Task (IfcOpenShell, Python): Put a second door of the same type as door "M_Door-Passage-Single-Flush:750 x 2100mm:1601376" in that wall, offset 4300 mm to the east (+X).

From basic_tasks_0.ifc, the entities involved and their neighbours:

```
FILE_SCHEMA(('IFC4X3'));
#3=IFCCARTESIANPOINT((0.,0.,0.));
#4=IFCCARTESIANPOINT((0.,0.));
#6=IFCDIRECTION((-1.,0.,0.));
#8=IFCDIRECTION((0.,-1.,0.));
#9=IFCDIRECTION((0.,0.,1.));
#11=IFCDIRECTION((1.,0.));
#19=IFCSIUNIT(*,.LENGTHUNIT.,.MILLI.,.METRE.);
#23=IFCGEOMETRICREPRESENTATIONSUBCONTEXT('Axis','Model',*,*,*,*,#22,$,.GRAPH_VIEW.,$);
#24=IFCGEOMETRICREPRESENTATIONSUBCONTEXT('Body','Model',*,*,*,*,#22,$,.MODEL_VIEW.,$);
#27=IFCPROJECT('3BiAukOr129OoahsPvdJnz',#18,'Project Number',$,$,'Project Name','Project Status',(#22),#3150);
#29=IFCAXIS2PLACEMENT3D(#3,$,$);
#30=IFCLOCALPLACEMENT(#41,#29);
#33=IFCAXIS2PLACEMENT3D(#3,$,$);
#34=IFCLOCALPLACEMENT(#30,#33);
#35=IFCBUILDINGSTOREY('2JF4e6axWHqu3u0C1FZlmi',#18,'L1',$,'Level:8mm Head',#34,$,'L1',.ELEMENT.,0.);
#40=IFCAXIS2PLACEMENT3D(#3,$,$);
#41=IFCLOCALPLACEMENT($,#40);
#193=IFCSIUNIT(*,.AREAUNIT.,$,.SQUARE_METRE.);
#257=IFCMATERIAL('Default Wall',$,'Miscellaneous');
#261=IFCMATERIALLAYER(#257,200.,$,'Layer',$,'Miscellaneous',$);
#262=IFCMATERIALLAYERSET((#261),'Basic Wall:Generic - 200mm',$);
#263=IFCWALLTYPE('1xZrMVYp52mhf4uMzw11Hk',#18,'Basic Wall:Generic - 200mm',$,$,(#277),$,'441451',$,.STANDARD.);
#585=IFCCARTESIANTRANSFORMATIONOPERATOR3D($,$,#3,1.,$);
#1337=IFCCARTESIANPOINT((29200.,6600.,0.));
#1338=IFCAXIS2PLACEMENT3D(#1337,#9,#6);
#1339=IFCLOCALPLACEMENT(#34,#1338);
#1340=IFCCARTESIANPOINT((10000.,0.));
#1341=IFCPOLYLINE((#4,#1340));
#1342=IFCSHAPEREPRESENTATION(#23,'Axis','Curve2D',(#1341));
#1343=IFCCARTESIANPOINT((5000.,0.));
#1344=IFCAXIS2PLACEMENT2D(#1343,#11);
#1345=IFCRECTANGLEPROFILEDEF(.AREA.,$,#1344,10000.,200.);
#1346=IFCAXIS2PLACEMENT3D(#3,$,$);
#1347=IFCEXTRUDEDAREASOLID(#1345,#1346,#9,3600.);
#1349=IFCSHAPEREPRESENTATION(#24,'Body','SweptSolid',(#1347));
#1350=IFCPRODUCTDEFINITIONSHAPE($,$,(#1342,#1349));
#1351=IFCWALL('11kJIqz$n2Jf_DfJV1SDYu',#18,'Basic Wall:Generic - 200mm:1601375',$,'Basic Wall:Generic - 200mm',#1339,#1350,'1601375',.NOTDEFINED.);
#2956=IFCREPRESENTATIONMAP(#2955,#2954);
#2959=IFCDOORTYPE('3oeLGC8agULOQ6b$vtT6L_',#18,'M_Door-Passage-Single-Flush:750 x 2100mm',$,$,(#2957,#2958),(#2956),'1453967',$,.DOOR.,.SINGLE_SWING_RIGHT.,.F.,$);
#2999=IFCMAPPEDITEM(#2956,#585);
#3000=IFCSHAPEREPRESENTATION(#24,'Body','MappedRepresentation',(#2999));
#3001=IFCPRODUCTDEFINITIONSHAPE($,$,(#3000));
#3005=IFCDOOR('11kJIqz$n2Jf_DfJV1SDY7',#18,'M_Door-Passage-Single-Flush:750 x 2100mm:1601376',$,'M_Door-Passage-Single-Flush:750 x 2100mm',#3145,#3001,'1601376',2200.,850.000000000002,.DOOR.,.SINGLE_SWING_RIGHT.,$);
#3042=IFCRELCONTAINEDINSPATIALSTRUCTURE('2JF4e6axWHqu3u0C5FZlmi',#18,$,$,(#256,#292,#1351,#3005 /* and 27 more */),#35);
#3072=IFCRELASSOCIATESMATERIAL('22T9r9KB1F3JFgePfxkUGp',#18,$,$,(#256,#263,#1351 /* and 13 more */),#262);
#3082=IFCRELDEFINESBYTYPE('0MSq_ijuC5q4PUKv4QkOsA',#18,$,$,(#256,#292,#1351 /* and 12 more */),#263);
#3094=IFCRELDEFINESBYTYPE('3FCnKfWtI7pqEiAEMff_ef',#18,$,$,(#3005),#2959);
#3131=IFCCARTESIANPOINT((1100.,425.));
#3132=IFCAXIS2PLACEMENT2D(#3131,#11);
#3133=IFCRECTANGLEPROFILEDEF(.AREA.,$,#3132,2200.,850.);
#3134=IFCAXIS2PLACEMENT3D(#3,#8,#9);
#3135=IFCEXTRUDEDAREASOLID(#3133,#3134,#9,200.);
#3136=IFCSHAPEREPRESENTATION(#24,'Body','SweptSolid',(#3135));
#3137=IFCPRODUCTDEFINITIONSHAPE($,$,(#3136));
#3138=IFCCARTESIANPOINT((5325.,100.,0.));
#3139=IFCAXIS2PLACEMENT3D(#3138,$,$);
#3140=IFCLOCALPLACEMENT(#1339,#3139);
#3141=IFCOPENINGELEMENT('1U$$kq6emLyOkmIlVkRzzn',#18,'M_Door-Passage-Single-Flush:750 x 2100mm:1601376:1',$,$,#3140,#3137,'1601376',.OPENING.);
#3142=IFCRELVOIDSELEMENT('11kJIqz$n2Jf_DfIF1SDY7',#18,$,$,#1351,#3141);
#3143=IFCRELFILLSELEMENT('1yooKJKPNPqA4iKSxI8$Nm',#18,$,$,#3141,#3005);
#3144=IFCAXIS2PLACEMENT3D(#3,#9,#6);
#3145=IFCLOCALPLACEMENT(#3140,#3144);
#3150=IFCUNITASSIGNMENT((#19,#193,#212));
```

```python
import ifcopenshell
import ifcopenshell.api.feature
import ifcopenshell.api.geometry
import ifcopenshell.api.root
import ifcopenshell.geom
import ifcopenshell.util.element
import ifcopenshell.util.placement
import ifcopenshell.util.shape

model = ifcopenshell.open("basic_tasks_0.ifc")
settings = ifcopenshell.geom.settings()


def volume(element):
    """Net volume in cubic metres, openings subtracted."""
    shape = ifcopenshell.geom.create_shape(settings, element)
    return ifcopenshell.util.shape.get_volume(shape.geometry)


def reuse_history(source, copy):
    """copy_class also copies each property set's owner history, people and application; keep the originals."""
    for rel in copy.IsDefinedBy:
        if rel.is_a("IfcRelDefinesByProperties") and (history := rel.RelatingPropertyDefinition.OwnerHistory):
            rel.RelatingPropertyDefinition.OwnerHistory = source.OwnerHistory
            ifcopenshell.util.element.remove_deep2(model, history)


door = model.by_id(3005)
opening = door.FillsVoids[0].RelatingOpeningElement
wall = opening.VoidsElements[0].RelatingBuildingElement
before = volume(wall)
shift = ifcopenshell.util.placement.get_local_placement(wall.ObjectPlacement)[:3, 0] * -4300.0

# copy_class copies the void relationship, type, container and properties, but no geometry.
new_opening = ifcopenshell.api.root.copy_class(model, product=opening)
new_opening.Representation = ifcopenshell.util.element.copy_deep(
    model, opening.Representation, exclude=["IfcGeometricRepresentationContext", "IfcRepresentationMap"]
)
new_opening.Name = "M_Door-Passage-Single-Flush:750 x 2100mm"
new_opening.Tag = None
new_door = ifcopenshell.api.root.copy_class(model, product=door)
new_door.Representation = ifcopenshell.util.element.copy_deep(
    model, door.Representation, exclude=["IfcGeometricRepresentationContext", "IfcRepresentationMap"]
)
new_door.Name = "M_Door-Passage-Single-Flush:750 x 2100mm"
new_door.Tag = None
reuse_history(door, new_door)
ifcopenshell.api.feature.add_filling(model, opening=new_opening, element=new_door)

for old, new in ((opening, new_opening), (door, new_door)):
    matrix = ifcopenshell.util.placement.get_local_placement(old.ObjectPlacement)
    matrix[:3, 3] += shift
    ifcopenshell.api.geometry.edit_object_placement(model, product=new, matrix=matrix, is_si=False)

after = volume(wall)

print(f"wall volume {before:.3f} -> {after:.3f} m3")

model.write("basic_tasks_0-out.ifc")
```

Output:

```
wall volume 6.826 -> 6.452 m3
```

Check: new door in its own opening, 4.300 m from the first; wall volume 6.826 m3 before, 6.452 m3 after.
